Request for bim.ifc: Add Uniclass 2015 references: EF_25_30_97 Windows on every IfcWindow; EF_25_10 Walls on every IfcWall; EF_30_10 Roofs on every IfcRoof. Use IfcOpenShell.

First a look at what the model holds.

```python
import ifcopenshell

model = ifcopenshell.open("bim.ifc")
print(model.schema)
print("classifications:", [c.Name for c in model.by_type("IfcClassification")])
for ifc_class in ("IfcDoor", "IfcRoof", "IfcStair", "IfcWall", "IfcWindow"):
    print(ifc_class, len(model.by_type(ifc_class)))
```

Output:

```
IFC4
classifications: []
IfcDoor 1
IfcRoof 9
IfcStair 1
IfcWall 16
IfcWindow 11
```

```python
import ifcopenshell
import ifcopenshell.api.classification

model = ifcopenshell.open("bim.ifc")

system = ifcopenshell.api.classification.add_classification(model, classification="Uniclass 2015")

codes = {
    "IfcWindow": ("EF_25_30_97", "Windows"),
    "IfcWall": ("EF_25_10", "Walls"),
    "IfcRoof": ("EF_30_10", "Roofs"),
}
for ifc_class, (code, name) in codes.items():
    products = model.by_type(ifc_class)
    ifcopenshell.api.classification.add_reference(
        model, products=products, classification=system, identification=code, name=name
    )
    print(code, len(products))

model.write("bim_edited.ifc")
```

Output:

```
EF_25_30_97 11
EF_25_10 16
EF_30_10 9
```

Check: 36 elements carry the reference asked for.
